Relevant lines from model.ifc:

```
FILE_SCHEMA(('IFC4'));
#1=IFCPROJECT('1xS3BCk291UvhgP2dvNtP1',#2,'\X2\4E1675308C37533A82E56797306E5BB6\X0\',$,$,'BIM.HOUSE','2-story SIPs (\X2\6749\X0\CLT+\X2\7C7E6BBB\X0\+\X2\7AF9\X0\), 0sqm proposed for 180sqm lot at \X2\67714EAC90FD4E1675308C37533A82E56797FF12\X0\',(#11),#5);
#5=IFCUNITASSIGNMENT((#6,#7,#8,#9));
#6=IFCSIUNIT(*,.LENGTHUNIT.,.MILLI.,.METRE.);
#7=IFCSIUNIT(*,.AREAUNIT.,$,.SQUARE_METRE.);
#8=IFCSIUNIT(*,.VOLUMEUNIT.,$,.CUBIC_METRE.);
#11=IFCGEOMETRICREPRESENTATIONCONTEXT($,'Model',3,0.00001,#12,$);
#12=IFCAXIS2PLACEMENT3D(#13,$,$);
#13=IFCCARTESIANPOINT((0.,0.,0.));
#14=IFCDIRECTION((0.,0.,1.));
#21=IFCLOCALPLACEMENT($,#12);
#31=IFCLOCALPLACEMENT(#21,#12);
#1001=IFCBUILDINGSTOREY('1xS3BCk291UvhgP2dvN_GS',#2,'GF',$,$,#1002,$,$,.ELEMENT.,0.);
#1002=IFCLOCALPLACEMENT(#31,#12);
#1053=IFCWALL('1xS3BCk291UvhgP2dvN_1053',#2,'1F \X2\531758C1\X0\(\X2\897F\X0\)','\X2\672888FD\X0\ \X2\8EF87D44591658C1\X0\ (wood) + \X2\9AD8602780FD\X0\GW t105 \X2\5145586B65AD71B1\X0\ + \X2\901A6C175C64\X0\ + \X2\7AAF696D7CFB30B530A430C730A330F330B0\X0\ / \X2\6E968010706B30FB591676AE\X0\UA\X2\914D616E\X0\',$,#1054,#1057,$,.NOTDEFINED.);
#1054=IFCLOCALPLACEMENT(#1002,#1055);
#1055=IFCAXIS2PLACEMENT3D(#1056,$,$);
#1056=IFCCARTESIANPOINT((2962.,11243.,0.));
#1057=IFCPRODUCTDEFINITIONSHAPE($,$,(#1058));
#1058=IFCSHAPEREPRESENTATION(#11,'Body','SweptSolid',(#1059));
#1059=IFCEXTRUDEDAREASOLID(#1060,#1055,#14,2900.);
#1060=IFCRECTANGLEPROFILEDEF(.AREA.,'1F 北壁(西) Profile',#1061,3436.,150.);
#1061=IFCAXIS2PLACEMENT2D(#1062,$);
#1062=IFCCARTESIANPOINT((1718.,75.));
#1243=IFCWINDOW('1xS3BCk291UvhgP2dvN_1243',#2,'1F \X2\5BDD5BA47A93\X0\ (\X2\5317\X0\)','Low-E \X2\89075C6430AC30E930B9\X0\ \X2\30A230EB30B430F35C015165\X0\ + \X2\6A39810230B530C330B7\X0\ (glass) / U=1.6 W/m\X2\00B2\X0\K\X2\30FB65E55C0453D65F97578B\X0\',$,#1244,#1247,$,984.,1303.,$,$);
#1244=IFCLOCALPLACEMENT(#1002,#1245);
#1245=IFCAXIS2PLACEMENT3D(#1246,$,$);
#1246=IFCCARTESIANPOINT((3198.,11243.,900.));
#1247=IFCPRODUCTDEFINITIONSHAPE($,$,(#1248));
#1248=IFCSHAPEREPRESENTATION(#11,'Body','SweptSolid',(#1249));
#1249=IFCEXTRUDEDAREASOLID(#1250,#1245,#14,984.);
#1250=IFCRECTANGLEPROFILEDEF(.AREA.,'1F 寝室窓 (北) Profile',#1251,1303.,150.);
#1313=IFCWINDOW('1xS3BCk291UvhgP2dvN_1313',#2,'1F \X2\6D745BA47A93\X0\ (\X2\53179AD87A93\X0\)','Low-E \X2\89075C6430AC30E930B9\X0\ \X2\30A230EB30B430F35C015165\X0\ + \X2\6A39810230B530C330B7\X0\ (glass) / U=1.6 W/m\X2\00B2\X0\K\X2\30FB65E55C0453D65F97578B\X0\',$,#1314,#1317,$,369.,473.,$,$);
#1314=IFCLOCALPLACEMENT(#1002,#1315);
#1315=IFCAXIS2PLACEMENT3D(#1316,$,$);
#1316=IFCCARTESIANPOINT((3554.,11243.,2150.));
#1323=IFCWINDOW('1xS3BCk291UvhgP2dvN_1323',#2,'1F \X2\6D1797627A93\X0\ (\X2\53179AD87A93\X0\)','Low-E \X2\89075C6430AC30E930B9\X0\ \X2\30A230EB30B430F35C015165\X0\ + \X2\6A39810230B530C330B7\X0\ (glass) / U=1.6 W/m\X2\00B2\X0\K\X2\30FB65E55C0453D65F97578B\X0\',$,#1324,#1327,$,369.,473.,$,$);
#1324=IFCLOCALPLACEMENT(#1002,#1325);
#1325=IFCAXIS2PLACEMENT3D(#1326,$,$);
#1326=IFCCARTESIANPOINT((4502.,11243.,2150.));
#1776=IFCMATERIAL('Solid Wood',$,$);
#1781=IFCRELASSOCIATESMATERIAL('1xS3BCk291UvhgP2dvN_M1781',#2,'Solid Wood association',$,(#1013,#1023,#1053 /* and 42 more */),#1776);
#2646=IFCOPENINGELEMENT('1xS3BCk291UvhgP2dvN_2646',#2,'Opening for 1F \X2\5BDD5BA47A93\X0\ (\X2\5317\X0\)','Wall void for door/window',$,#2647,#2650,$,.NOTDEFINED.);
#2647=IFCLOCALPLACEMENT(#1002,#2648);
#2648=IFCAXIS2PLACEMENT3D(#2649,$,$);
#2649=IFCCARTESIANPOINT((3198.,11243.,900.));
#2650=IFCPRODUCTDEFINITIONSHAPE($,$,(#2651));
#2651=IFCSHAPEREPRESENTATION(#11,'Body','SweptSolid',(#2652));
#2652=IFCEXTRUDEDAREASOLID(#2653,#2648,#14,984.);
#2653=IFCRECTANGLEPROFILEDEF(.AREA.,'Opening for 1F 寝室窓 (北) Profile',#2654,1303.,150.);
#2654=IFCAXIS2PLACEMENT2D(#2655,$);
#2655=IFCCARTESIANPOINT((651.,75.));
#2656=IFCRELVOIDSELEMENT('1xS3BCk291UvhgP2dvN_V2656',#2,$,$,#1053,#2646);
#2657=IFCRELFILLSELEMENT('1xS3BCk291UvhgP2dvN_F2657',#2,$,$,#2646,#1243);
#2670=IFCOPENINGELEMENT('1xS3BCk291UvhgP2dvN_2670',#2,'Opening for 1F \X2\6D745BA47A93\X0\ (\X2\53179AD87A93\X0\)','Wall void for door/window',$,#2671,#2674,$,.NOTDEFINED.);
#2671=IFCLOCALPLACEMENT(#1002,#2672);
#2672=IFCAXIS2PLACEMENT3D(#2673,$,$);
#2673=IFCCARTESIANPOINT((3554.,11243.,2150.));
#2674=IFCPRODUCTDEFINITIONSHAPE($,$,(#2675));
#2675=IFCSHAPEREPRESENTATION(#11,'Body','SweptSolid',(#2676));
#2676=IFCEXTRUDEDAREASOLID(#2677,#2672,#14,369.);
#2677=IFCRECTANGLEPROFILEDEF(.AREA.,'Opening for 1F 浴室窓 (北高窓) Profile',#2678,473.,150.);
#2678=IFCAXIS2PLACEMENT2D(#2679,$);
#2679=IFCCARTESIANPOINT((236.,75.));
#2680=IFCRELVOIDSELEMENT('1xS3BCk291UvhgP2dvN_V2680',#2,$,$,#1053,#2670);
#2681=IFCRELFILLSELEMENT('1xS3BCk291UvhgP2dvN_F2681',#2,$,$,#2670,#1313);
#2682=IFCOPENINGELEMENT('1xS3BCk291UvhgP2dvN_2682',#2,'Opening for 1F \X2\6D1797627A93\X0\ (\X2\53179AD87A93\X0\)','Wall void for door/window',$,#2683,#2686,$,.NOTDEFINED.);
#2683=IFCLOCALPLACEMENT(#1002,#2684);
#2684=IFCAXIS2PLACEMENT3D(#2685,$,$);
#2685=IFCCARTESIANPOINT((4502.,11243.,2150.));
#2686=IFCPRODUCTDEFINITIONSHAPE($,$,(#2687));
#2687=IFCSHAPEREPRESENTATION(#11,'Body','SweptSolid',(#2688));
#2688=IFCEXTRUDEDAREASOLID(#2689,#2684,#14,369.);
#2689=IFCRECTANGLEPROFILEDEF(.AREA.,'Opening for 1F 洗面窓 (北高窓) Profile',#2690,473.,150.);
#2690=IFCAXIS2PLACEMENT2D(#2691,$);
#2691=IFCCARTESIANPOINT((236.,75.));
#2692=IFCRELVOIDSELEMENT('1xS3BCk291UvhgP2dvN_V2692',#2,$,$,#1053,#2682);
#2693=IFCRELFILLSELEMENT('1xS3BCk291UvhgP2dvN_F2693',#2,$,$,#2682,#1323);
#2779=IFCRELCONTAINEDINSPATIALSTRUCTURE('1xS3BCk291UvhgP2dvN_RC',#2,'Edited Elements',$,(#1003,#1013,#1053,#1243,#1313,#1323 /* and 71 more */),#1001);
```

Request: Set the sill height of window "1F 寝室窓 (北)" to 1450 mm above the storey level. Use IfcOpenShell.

```python
import numpy as np
import ifcopenshell
import ifcopenshell.api.geometry
import ifcopenshell.geom
import ifcopenshell.util.element
import ifcopenshell.util.placement
import ifcopenshell.util.shape
import ifcopenshell.util.unit

model = ifcopenshell.open("model.ifc")
unit_scale = ifcopenshell.util.unit.calculate_unit_scale(model)

window = model.by_guid("1xS3BCk291UvhgP2dvN_1243")
opening = window.FillsVoids[0].RelatingOpeningElement
storey = ifcopenshell.util.element.get_container(window, ifc_class="IfcBuildingStorey")
level = ifcopenshell.util.placement.get_local_placement(storey.ObjectPlacement)[2, 3]

# The opening's origin need not be at the sill, so measure its lowest point.
shape = ifcopenshell.geom.create_shape(ifcopenshell.geom.settings(), opening)
bottom = ifcopenshell.util.shape.get_shape_bottom_elevation(shape, shape.geometry) / unit_scale
dz = level + 1.45 / unit_scale - bottom

shift = np.array([0.0, 0.0, dz])
# The window is not placed relative to its opening, so move both.
for product in (opening, window):
    matrix = ifcopenshell.util.placement.get_local_placement(product.ObjectPlacement)
    matrix[:3, 3] += shift
    ifcopenshell.api.geometry.edit_object_placement(model, product=product, matrix=matrix, is_si=False)

print(f"moved by {dz * unit_scale:+.3f} m")

model.write("model_v2.ifc")
```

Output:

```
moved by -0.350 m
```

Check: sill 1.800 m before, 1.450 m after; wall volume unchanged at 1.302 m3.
